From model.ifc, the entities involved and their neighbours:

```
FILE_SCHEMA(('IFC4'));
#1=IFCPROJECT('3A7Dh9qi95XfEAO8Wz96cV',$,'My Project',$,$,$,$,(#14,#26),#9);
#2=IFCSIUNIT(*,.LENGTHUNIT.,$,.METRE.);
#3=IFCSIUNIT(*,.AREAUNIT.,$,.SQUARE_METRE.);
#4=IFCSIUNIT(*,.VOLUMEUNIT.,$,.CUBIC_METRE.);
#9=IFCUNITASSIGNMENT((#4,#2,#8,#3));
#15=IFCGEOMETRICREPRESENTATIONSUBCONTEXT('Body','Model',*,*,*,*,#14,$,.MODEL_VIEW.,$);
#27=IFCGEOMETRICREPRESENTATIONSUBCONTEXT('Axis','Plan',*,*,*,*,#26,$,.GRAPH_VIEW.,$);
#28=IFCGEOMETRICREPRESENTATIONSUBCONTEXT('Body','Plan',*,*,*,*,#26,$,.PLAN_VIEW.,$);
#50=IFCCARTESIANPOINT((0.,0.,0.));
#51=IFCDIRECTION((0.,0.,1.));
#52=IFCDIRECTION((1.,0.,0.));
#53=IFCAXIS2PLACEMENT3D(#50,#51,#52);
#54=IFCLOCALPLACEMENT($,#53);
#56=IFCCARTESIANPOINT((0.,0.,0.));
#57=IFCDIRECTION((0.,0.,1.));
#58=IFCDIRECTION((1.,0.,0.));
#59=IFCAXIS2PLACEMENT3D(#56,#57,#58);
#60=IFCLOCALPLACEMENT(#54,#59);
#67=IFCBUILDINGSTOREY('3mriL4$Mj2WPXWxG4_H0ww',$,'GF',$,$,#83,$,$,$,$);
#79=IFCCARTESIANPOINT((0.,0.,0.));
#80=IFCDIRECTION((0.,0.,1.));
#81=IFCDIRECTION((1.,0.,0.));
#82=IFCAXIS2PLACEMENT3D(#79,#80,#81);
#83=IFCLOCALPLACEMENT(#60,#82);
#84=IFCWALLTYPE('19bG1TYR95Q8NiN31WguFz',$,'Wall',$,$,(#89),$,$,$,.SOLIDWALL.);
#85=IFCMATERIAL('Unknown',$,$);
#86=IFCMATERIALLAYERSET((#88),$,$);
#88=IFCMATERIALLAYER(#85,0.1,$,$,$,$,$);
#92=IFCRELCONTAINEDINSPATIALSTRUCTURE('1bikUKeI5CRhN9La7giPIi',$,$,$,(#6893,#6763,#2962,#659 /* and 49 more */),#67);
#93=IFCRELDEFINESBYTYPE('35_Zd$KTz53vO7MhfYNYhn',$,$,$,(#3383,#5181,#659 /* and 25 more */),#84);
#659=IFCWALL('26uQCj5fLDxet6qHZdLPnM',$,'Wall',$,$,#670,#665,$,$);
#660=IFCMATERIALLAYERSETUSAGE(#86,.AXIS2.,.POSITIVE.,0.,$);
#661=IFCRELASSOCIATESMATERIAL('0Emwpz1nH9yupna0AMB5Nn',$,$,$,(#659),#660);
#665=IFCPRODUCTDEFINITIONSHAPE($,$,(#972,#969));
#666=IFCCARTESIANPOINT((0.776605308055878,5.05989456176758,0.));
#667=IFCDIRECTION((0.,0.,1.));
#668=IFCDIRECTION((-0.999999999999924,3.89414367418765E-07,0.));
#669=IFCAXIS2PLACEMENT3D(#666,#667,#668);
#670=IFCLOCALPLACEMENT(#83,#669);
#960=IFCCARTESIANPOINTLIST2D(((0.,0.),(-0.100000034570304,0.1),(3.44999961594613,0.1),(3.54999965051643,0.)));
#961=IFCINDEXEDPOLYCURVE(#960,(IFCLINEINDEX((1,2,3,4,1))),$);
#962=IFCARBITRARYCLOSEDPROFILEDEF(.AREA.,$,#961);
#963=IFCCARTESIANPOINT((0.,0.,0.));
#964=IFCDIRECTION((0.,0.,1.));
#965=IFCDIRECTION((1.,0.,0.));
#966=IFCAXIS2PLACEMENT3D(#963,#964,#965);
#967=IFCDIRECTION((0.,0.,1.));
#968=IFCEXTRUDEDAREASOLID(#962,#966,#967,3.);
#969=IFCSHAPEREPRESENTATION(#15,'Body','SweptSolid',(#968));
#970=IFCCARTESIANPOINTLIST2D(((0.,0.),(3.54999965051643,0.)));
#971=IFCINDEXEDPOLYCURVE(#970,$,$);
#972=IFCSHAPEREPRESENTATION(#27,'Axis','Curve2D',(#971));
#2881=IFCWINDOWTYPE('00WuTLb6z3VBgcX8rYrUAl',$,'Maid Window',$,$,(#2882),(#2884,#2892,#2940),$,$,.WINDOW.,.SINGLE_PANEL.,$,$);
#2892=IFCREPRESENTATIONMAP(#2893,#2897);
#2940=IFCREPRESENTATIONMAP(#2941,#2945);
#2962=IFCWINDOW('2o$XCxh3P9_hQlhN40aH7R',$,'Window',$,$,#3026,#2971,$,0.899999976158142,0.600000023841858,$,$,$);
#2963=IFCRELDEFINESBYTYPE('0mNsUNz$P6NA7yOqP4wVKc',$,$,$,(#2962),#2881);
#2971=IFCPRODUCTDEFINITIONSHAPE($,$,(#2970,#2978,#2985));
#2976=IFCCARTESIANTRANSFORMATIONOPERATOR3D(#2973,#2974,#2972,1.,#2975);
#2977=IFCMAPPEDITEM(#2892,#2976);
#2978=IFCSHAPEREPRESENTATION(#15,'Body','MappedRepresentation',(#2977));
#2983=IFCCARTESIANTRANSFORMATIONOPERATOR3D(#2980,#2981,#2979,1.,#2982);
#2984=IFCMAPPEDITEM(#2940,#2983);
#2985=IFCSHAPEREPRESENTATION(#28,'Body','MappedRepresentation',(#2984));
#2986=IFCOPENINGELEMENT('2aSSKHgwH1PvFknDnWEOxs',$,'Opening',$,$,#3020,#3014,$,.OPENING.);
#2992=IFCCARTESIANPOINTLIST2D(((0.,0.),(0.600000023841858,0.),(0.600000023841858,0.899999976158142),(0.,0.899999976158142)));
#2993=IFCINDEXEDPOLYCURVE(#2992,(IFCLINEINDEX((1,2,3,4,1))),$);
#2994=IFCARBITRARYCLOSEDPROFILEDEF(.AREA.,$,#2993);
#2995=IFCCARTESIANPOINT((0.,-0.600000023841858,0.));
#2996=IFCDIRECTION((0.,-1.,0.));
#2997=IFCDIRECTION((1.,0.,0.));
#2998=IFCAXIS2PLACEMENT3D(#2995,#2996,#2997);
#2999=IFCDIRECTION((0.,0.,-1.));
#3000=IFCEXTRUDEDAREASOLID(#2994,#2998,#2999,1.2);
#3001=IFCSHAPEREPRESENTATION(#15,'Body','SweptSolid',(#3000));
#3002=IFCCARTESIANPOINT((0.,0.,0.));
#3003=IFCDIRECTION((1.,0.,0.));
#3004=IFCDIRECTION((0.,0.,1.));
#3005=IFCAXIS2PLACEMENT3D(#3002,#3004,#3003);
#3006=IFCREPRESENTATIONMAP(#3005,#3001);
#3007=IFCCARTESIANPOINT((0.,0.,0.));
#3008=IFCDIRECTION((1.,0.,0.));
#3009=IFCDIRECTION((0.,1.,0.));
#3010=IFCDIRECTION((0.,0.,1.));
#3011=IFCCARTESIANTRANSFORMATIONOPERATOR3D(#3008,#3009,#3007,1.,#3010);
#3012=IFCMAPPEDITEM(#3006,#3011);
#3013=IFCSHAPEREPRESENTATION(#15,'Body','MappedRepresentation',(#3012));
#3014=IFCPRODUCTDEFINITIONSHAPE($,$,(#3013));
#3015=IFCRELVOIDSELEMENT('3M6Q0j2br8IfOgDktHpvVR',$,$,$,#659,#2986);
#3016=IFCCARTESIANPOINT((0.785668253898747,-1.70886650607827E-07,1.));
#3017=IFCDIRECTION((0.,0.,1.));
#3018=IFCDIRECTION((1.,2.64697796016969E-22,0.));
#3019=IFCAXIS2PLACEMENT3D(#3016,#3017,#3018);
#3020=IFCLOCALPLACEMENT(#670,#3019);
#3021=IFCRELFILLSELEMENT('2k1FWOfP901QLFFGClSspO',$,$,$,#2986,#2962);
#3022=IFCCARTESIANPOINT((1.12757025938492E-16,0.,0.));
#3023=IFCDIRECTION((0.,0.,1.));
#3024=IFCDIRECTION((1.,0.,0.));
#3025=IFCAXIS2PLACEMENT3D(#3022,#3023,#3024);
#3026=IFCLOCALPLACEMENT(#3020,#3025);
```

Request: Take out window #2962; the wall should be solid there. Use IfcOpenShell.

```python
import ifcopenshell
import ifcopenshell.api.feature
import ifcopenshell.api.root
import ifcopenshell.geom
import ifcopenshell.util.shape

model = ifcopenshell.open("model.ifc")
settings = ifcopenshell.geom.settings()


def volume(element):
    """Net volume in cubic metres, openings subtracted."""
    shape = ifcopenshell.geom.create_shape(settings, element)
    return ifcopenshell.util.shape.get_volume(shape.geometry)


window = model.by_id(2962)
opening = window.FillsVoids[0].RelatingOpeningElement
wall = opening.VoidsElements[0].RelatingBuildingElement
before = volume(wall)

ifcopenshell.api.root.remove_product(model, product=window)
ifcopenshell.api.feature.remove_feature(model, feature=opening)

after = volume(wall)

print(f"wall volume {before:.3f} -> {after:.3f} m3")

model.write("model_updated.ifc")
```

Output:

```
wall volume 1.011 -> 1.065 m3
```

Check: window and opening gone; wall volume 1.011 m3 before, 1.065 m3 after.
